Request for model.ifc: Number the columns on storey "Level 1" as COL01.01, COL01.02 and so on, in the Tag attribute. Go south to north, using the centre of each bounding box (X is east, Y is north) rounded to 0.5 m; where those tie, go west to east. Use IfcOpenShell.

First a look at what the model holds.

```python
import ifcopenshell
import ifcopenshell.util.element
import ifcopenshell.util.placement

model = ifcopenshell.open("model.ifc")
print(model.schema)
storey = next(s for s in model.by_type("IfcBuildingStorey") if s.Name == "Level 1")
columns = [e for e in ifcopenshell.util.element.get_decomposition(storey) if e.is_a("IfcColumn")]
for e in sorted(columns, key=lambda e: e.id()):
    origin = ifcopenshell.util.placement.get_local_placement(e.ObjectPlacement)[:3, 3]
    print(e.id(), e.Tag, e.Name, origin.round(2) + 0.0, sep=" | ")
```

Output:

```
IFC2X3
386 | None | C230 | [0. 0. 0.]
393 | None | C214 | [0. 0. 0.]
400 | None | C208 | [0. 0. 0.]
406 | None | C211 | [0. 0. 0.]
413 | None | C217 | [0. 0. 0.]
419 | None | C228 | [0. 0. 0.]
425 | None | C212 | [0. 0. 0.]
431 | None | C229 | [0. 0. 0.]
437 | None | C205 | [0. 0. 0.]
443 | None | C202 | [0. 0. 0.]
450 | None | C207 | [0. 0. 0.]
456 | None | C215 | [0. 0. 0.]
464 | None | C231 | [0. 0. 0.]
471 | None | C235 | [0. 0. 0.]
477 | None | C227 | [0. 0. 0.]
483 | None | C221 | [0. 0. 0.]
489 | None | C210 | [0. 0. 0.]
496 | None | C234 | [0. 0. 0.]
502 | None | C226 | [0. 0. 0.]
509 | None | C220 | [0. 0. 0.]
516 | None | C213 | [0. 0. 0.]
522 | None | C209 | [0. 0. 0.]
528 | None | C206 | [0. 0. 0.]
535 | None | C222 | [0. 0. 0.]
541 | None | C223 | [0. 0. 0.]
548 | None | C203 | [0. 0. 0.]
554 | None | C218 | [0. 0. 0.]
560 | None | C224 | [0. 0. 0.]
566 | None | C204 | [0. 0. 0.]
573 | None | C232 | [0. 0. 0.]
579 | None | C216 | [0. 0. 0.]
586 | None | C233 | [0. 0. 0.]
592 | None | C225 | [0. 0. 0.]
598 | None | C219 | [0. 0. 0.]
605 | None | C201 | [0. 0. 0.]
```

```python
import ifcopenshell
import ifcopenshell.geom
import ifcopenshell.util.element
import ifcopenshell.util.shape

model = ifcopenshell.open("model.ifc")
settings = ifcopenshell.geom.settings()
settings.set("use-world-coords", True)


def centre(element):
    shape = ifcopenshell.geom.create_shape(settings, element)
    return ifcopenshell.util.shape.get_bbox_centroid(shape.geometry)


storey = next(s for s in model.by_type("IfcBuildingStorey") if s.Name == "Level 1")
columns = [e for e in ifcopenshell.util.element.get_decomposition(storey) if e.is_a("IfcColumn")]

# Insertion points can sit at a corner or the storey origin, so sort by the geometry (in metres).
centres = {e: centre(e) for e in columns}
columns.sort(key=lambda e: (round(centres[e][1] / 0.5), centres[e][0]))

for i, e in enumerate(columns, start=1):
    number = f"COL01.{i:02d}"
    e.Tag = number
    print(e.id(), number)

model.write("model_updated.ifc")
```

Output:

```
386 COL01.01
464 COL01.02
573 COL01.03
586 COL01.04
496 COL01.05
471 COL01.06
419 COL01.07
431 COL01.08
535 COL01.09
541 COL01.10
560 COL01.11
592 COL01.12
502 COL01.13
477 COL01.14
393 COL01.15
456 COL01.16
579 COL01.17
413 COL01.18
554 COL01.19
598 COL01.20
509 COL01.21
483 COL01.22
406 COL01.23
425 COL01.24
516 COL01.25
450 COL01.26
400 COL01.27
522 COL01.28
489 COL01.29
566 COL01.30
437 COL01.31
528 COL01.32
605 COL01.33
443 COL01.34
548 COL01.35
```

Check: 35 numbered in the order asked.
